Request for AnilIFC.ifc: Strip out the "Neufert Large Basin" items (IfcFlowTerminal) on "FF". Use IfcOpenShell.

First a look at what the model holds.

```python
import ifcopenshell
import ifcopenshell.util.element

model = ifcopenshell.open("AnilIFC.ifc")
print(model.schema)
storey = next(s for s in model.by_type("IfcBuildingStorey") if s.Name == "FF")
terminals = [e for e in ifcopenshell.util.element.get_decomposition(storey) if e.is_a("IfcFlowTerminal")]
seen = {}
for e in terminals:
    element_type = ifcopenshell.util.element.get_type(e)
    name = element_type.Name if element_type not in (None, e) else None
    seen[name] = seen.get(name, 0) + 1
for name, count in sorted(seen.items(), key=str):
    print(count, "x", name)
```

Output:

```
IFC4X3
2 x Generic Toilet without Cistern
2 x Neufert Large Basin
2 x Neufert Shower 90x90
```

```python
import ifcopenshell
import ifcopenshell.api.root
import ifcopenshell.util.element

model = ifcopenshell.open("AnilIFC.ifc")

storey = next(s for s in model.by_type("IfcBuildingStorey") if s.Name == "FF")
terminals = [e for e in ifcopenshell.util.element.get_decomposition(storey) if e.is_a("IfcFlowTerminal")]
targets = [e for e in terminals if (t := ifcopenshell.util.element.get_type(e)) not in (None, e) and t.Name == "Neufert Large Basin"]

for e in targets:
    ifcopenshell.api.root.remove_product(model, product=e)
print(len(targets), "removed")

model.write("AnilIFC_rev.ifc")
```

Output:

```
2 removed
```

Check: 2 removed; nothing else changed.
